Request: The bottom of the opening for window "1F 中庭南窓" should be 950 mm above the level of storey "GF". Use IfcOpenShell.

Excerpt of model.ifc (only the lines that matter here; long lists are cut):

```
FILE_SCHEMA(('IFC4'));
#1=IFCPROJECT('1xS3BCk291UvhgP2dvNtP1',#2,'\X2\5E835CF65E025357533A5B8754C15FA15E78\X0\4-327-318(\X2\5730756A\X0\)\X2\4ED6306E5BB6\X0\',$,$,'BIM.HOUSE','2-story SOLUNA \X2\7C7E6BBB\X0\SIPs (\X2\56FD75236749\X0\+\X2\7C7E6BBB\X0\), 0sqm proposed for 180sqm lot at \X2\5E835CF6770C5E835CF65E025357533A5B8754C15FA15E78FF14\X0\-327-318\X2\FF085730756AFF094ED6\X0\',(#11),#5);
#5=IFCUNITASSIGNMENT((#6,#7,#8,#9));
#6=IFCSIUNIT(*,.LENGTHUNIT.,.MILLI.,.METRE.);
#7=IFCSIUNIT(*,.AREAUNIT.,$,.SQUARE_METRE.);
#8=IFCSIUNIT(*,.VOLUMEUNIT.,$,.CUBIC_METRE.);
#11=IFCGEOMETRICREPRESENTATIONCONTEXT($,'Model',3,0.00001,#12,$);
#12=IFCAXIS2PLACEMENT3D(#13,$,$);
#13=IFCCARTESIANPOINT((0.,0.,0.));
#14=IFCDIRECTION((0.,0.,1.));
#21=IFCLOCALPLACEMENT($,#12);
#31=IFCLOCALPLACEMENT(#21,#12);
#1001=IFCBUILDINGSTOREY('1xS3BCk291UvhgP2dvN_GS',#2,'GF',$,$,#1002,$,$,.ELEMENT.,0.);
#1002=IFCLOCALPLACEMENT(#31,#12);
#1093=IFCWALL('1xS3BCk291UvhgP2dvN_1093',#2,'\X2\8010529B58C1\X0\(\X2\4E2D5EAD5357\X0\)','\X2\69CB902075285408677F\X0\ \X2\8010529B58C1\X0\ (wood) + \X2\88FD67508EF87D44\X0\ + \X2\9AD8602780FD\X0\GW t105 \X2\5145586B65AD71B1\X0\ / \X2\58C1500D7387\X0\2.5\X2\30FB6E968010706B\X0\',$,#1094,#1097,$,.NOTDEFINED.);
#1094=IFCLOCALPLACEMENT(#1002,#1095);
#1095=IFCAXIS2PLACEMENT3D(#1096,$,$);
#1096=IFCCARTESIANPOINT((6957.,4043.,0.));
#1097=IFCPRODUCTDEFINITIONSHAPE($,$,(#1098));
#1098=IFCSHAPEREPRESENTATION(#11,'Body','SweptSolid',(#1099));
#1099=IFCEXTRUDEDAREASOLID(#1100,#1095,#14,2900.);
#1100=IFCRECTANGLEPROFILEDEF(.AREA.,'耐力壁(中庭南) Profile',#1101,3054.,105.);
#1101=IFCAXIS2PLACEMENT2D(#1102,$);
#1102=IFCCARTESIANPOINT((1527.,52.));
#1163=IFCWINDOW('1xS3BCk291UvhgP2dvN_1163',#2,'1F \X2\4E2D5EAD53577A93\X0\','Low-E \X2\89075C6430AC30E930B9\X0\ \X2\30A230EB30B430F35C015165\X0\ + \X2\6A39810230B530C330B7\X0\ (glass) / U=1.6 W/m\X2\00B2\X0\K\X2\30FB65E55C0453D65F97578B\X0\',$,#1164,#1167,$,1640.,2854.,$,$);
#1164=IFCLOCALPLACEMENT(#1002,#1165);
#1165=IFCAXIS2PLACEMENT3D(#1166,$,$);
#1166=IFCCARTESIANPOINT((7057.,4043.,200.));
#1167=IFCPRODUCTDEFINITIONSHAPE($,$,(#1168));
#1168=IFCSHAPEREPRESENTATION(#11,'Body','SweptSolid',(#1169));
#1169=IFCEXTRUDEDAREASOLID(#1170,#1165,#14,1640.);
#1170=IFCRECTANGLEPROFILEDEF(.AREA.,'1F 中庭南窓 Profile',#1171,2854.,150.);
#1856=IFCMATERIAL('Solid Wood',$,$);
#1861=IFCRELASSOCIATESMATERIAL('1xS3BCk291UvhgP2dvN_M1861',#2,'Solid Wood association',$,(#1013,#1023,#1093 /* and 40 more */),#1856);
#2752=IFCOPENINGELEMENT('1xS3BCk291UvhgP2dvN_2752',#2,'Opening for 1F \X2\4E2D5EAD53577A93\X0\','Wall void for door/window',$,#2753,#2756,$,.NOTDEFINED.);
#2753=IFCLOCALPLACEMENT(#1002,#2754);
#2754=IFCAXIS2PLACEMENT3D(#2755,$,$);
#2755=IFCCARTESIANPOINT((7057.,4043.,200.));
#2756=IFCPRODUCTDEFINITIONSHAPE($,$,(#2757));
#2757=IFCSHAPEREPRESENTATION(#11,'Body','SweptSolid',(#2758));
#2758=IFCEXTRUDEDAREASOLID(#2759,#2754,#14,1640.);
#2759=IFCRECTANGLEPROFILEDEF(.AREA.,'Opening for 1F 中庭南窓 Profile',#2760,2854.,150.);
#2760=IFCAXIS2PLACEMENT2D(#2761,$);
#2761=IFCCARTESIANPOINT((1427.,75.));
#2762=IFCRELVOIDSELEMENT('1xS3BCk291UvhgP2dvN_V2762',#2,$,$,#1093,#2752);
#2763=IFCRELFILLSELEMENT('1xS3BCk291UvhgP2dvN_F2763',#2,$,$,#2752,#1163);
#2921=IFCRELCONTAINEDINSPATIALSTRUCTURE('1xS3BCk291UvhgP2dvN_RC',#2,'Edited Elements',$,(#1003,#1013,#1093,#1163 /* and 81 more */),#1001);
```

```python
import numpy as np
import ifcopenshell
import ifcopenshell.api.geometry
import ifcopenshell.geom
import ifcopenshell.util.element
import ifcopenshell.util.placement
import ifcopenshell.util.shape
import ifcopenshell.util.unit

model = ifcopenshell.open("model.ifc")
unit_scale = ifcopenshell.util.unit.calculate_unit_scale(model)

window = model.by_id(1163)
opening = window.FillsVoids[0].RelatingOpeningElement
storey = ifcopenshell.util.element.get_container(window, ifc_class="IfcBuildingStorey")
level = ifcopenshell.util.placement.get_local_placement(storey.ObjectPlacement)[2, 3]

# The opening's origin need not be at the sill, so measure its lowest point.
shape = ifcopenshell.geom.create_shape(ifcopenshell.geom.settings(), opening)
bottom = ifcopenshell.util.shape.get_shape_bottom_elevation(shape, shape.geometry) / unit_scale
dz = level + 950.0 - bottom

shift = np.array([0.0, 0.0, dz])
# The window is not placed relative to its opening, so move both.
for product in (opening, window):
    matrix = ifcopenshell.util.placement.get_local_placement(product.ObjectPlacement)
    matrix[:3, 3] += shift
    ifcopenshell.api.geometry.edit_object_placement(model, product=product, matrix=matrix, is_si=False)

print(f"moved by {dz * unit_scale:+.3f} m")

model.write("model_rev.ifc")
```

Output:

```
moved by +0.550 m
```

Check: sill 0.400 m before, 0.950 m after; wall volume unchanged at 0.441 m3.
